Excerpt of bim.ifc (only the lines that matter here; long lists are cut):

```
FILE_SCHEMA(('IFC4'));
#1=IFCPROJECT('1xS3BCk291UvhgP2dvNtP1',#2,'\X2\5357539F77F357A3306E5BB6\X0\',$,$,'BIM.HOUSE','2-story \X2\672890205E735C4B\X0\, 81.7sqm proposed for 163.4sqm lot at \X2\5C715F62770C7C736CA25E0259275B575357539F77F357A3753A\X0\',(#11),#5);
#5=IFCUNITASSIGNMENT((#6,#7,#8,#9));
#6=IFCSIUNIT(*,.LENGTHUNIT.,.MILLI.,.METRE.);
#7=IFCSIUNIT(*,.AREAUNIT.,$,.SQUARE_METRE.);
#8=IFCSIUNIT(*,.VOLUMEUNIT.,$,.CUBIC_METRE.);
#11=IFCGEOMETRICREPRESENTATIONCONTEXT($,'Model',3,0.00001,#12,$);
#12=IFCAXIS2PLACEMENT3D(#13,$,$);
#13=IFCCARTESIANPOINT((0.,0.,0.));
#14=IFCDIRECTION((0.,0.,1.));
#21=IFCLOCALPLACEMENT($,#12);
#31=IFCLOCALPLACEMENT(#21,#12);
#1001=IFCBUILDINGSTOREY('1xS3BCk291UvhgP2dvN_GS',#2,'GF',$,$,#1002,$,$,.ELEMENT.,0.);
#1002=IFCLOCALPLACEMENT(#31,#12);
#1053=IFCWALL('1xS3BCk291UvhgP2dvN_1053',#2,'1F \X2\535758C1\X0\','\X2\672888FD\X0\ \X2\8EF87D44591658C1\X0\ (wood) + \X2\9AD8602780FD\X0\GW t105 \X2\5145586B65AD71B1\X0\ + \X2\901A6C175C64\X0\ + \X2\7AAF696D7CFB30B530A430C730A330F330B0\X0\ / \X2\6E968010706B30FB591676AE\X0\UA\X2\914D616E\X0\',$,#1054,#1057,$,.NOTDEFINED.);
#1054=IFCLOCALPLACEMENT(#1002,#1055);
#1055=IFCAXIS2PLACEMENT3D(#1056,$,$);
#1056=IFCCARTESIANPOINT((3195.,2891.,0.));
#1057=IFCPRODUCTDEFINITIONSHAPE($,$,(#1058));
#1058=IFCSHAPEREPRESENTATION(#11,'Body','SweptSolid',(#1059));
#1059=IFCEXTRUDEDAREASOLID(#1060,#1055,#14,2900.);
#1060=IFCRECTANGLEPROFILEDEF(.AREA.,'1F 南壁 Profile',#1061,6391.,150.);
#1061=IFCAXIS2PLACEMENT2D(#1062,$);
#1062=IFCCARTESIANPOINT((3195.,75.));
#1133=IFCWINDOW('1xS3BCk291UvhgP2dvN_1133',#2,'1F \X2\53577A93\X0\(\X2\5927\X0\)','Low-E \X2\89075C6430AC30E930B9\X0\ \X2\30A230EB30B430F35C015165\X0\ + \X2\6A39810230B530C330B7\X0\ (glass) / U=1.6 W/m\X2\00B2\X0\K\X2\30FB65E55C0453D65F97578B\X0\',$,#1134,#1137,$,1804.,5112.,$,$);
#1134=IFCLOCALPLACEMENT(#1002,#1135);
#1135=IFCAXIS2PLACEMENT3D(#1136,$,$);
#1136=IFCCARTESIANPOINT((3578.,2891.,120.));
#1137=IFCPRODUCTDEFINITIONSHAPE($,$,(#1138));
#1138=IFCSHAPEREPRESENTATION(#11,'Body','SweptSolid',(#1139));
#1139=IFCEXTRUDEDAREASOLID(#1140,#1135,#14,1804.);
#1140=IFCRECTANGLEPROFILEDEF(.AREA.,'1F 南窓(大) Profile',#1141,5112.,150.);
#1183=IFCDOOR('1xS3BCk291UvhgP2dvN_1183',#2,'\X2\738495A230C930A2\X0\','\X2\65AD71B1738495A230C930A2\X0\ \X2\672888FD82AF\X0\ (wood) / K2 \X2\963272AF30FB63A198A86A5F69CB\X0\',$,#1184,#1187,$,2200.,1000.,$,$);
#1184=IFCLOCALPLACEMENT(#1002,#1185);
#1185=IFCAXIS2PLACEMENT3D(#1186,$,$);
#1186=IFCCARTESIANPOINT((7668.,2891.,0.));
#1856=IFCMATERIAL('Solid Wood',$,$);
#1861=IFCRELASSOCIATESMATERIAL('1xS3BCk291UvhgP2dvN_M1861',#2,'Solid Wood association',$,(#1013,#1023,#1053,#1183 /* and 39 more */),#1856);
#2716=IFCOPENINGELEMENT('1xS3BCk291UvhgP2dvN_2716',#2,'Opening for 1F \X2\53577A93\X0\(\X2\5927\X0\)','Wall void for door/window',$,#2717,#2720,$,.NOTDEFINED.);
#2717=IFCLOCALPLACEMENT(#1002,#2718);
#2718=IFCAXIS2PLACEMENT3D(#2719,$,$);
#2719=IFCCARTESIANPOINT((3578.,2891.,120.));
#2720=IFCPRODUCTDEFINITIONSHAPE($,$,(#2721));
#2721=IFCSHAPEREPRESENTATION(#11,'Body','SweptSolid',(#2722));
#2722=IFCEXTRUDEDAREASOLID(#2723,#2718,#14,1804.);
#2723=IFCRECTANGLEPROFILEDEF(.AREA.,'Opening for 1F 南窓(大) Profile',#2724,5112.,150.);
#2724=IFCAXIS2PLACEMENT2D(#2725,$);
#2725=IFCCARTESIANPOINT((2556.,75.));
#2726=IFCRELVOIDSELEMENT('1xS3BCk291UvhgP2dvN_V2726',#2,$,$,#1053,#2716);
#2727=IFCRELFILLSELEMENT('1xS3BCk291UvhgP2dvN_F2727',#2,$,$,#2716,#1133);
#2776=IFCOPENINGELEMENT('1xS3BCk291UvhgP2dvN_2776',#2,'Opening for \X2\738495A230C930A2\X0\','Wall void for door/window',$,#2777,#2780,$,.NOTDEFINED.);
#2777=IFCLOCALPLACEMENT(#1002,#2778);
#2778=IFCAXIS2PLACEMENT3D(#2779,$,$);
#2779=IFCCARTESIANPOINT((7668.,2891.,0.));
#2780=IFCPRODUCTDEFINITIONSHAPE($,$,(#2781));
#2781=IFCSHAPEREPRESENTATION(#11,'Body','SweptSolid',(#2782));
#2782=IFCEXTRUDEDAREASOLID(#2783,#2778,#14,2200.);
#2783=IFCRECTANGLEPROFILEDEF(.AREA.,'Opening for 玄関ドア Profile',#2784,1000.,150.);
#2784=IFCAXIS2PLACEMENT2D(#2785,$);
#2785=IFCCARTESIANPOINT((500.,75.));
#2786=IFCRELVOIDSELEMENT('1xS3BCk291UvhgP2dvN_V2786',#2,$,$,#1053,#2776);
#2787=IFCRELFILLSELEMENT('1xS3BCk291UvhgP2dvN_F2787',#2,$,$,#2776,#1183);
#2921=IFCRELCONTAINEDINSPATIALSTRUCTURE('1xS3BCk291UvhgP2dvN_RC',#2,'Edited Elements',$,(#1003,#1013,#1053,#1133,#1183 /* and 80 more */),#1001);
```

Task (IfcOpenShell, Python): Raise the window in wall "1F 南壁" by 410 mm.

```python
import numpy as np
import ifcopenshell
import ifcopenshell.api.geometry
import ifcopenshell.util.placement
import ifcopenshell.util.unit

model = ifcopenshell.open("bim.ifc")
unit_scale = ifcopenshell.util.unit.calculate_unit_scale(model)

window = model.by_guid("1xS3BCk291UvhgP2dvN_1133")
opening = window.FillsVoids[0].RelatingOpeningElement
dz = 0.41 / unit_scale

shift = np.array([0.0, 0.0, dz])
# The window is not placed relative to its opening, so move both.
for product in (opening, window):
    matrix = ifcopenshell.util.placement.get_local_placement(product.ObjectPlacement)
    matrix[:3, 3] += shift
    ifcopenshell.api.geometry.edit_object_placement(model, product=product, matrix=matrix, is_si=False)

print(f"moved by {dz * unit_scale:+.3f} m")

model.write("bim_rev.ifc")
```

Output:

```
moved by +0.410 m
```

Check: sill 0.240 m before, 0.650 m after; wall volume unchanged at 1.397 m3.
